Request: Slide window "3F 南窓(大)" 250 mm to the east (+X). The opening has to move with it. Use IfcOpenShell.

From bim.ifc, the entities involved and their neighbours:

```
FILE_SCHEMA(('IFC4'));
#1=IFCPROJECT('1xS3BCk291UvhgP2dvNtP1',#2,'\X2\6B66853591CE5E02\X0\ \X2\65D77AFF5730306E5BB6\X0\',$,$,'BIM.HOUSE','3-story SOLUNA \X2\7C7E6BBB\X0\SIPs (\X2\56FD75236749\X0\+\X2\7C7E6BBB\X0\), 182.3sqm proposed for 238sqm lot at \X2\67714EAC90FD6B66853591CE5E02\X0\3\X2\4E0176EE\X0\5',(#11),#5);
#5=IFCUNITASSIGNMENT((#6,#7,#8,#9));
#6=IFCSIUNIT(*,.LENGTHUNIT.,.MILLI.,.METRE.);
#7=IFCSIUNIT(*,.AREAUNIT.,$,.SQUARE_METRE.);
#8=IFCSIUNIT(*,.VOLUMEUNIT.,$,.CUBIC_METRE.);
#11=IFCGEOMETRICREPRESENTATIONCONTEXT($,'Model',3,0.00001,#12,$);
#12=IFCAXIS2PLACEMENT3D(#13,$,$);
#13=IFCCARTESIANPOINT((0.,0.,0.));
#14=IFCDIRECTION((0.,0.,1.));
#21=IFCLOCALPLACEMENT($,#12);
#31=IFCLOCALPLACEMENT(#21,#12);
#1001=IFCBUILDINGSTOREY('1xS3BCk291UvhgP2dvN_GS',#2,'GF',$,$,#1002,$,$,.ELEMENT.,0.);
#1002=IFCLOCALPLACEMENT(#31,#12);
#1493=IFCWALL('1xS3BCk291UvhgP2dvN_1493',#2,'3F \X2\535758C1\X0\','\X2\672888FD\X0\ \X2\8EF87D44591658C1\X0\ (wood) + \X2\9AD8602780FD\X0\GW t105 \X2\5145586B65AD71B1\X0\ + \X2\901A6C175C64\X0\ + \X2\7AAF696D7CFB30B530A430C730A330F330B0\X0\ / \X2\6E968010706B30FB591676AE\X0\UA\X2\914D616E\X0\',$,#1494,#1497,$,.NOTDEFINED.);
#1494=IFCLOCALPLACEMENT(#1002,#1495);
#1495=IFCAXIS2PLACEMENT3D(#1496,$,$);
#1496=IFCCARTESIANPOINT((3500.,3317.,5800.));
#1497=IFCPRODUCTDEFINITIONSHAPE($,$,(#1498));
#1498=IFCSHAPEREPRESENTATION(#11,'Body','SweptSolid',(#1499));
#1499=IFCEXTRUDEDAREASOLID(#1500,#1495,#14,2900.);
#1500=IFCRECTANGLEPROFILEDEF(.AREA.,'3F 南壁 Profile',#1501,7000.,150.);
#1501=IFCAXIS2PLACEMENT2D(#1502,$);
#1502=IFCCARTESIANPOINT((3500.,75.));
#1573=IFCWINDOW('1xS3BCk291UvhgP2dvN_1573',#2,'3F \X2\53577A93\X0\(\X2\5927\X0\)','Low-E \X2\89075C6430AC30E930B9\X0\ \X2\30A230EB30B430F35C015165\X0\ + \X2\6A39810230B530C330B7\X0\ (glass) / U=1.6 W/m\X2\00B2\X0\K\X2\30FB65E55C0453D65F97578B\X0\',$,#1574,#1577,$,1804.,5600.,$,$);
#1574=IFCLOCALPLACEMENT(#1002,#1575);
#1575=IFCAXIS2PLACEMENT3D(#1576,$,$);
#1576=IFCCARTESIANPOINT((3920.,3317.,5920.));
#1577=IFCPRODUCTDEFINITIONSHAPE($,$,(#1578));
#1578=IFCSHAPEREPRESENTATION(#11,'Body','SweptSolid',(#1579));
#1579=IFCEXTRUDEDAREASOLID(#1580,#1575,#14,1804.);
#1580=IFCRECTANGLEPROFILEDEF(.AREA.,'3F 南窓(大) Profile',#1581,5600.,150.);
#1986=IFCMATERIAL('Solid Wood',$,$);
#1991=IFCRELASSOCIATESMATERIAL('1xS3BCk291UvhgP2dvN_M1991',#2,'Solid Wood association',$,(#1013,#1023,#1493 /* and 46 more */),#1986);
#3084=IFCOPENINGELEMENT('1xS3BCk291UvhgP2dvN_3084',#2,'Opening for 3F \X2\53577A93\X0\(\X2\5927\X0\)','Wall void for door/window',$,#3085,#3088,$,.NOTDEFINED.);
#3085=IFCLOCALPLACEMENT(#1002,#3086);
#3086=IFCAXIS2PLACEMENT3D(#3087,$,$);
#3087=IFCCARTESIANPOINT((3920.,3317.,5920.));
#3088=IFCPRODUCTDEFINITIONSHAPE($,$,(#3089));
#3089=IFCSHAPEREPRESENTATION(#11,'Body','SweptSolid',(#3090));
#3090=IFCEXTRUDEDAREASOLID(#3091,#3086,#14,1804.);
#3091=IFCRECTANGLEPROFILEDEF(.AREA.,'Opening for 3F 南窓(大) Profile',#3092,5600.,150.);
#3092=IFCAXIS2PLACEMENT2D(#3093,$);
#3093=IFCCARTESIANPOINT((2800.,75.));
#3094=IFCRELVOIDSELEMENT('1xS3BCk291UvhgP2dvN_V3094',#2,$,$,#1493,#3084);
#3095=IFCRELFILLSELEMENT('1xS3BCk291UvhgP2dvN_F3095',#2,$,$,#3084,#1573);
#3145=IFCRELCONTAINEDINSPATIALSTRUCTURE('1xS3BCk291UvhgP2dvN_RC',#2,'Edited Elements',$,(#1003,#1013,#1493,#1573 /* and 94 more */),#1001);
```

```python
import ifcopenshell
import ifcopenshell.api.geometry
import ifcopenshell.util.placement
import ifcopenshell.util.unit

model = ifcopenshell.open("bim.ifc")
unit_scale = ifcopenshell.util.unit.calculate_unit_scale(model)

window = model.by_id(1573)
opening = window.FillsVoids[0].RelatingOpeningElement
wall = opening.VoidsElements[0].RelatingBuildingElement

wall_matrix = ifcopenshell.util.placement.get_local_placement(wall.ObjectPlacement)
shift = wall_matrix[:3, 0] * 0.25 / unit_scale
before = ifcopenshell.util.placement.get_local_placement(window.ObjectPlacement)[:3, 3].copy()

# The window is not placed relative to its opening, so move both.
for product in (opening, window):
    matrix = ifcopenshell.util.placement.get_local_placement(product.ObjectPlacement)
    matrix[:3, 3] += shift
    ifcopenshell.api.geometry.edit_object_placement(model, product=product, matrix=matrix, is_si=False)

after = ifcopenshell.util.placement.get_local_placement(window.ObjectPlacement)[:3, 3]
print("window moved by", (after - before).round(3) + 0.0)

model.write("bim_rev.ifc")
```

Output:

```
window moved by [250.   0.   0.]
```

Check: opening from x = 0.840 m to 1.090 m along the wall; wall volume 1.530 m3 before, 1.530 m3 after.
